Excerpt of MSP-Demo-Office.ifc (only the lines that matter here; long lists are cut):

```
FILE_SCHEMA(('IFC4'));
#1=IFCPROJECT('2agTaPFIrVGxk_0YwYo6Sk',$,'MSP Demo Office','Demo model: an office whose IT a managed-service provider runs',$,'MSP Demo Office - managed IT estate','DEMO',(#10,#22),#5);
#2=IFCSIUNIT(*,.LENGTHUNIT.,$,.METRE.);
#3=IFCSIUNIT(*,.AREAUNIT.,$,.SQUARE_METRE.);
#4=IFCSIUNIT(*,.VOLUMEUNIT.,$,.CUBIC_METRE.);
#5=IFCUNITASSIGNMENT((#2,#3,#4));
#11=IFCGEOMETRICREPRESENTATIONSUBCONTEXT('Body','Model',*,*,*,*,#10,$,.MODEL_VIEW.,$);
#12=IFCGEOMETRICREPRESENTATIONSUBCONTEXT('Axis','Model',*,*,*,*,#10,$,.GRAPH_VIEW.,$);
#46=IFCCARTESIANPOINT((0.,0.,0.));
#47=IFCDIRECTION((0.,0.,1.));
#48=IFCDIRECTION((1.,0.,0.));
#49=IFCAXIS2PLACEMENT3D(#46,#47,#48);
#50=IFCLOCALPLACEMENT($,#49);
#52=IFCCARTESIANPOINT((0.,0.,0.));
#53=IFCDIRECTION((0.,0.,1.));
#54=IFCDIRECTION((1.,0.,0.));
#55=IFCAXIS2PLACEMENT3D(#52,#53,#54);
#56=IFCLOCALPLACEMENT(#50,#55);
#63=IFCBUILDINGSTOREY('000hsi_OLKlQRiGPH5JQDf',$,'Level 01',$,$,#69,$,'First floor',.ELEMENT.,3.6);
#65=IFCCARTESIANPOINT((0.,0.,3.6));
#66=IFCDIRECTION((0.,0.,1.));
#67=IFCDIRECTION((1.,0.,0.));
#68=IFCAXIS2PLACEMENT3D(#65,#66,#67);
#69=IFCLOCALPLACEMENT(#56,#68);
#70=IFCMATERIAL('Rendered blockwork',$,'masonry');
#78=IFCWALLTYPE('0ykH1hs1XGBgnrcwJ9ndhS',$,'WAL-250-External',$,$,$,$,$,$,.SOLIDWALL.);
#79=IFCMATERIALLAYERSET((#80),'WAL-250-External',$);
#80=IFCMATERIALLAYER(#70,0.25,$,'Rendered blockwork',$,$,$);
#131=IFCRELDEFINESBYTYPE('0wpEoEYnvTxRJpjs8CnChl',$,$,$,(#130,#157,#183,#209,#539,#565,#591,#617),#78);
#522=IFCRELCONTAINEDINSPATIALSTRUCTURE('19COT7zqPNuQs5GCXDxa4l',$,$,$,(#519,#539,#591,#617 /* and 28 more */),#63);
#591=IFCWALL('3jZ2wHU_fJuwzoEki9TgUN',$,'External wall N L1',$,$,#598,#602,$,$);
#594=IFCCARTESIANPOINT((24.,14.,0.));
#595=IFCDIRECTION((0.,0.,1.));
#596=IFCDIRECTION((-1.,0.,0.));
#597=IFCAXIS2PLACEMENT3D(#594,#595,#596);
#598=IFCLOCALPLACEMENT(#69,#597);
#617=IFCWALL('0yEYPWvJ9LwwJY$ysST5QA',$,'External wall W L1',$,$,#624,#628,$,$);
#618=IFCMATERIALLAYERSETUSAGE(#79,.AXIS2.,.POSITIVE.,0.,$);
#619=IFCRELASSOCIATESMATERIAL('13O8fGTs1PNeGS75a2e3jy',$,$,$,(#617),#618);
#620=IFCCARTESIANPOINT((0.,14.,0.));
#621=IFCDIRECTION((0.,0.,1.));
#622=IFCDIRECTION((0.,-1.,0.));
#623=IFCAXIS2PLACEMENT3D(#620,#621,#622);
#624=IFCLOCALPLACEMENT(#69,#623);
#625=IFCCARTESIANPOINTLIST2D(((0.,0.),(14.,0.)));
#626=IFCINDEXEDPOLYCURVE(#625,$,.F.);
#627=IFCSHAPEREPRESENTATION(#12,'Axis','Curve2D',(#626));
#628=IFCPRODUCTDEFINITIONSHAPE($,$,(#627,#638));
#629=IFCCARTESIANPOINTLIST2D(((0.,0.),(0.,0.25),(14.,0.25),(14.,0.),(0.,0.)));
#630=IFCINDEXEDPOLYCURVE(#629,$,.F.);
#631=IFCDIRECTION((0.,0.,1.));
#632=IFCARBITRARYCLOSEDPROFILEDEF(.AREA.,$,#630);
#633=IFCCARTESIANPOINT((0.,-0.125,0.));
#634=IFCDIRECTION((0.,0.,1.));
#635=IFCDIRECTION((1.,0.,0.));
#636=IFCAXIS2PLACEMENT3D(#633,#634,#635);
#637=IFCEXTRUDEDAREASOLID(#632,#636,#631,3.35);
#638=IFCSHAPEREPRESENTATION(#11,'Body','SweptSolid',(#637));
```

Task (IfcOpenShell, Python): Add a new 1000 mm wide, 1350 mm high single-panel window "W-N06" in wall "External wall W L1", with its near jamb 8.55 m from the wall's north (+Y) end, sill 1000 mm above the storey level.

```python
import numpy as np
import ifcopenshell
import ifcopenshell.api.feature
import ifcopenshell.api.geometry
import ifcopenshell.api.root
import ifcopenshell.api.spatial
import ifcopenshell.geom
import ifcopenshell.util.element
import ifcopenshell.util.placement
import ifcopenshell.util.representation
import ifcopenshell.util.shape
import ifcopenshell.util.unit

model = ifcopenshell.open("MSP-Demo-Office.ifc")
unit_scale = ifcopenshell.util.unit.calculate_unit_scale(model)
settings = ifcopenshell.geom.settings()


def volume(element):
    """Net volume in cubic metres, openings subtracted."""
    shape = ifcopenshell.geom.create_shape(settings, element)
    return ifcopenshell.util.shape.get_volume(shape.geometry)


wall = model.by_guid("0yEYPWvJ9LwwJY$ysST5QA")
storey = ifcopenshell.util.element.get_container(wall, ifc_class="IfcBuildingStorey")
context = ifcopenshell.util.representation.get_context(model, "Model", "Body", "MODEL_VIEW")
before = volume(wall)

width, height, from_end, sill = 1, 1.35, 8.55, 1  # metres

# The wall runs along its own X axis, and the end named is its -X end.
wall_shape = ifcopenshell.geom.create_shape(settings, wall)
x, y, z = ifcopenshell.util.shape.get_vertices(wall_shape.geometry).T
start = x.min() + from_end
face, thickness = float(y.min()), float(y.max() - y.min())
wall_matrix = ifcopenshell.util.placement.get_local_placement(wall.ObjectPlacement)
level = ifcopenshell.util.placement.get_local_placement(storey.ObjectPlacement)[2, 3]


def in_wall(x, y):
    """Placement at x, y metres in the wall's axes, at sill height."""
    matrix = wall_matrix.copy()
    matrix[:, 3] = wall_matrix @ np.array([x / unit_scale, y / unit_scale, 0.0, 1.0])
    matrix[2, 3] = level + sill / unit_scale
    return matrix


# Opening: a box that overshoots both wall faces by 50 mm.
opening = ifcopenshell.api.root.create_entity(model, ifc_class="IfcOpeningElement", predefined_type="OPENING")
box = ifcopenshell.api.geometry.add_wall_representation(
    model, context=context, length=width, height=height, thickness=thickness + 0.1
)
ifcopenshell.api.geometry.assign_representation(model, product=opening, representation=box)
ifcopenshell.api.geometry.edit_object_placement(model, product=opening, matrix=in_wall(start, face - 0.05), is_si=False)
ifcopenshell.api.feature.add_feature(model, feature=opening, element=wall)

window = ifcopenshell.api.root.create_entity(model, ifc_class="IfcWindow", name="W-N06", predefined_type="WINDOW")
window.OverallWidth, window.OverallHeight = width / unit_scale, height / unit_scale
window.PartitioningType = "SINGLE_PANEL"
body = ifcopenshell.api.geometry.add_window_representation(
    model,
    context=context,
    overall_width=window.OverallWidth,
    overall_height=window.OverallHeight,
    partition_type="SINGLE_PANEL",
)
ifcopenshell.api.geometry.assign_representation(model, product=window, representation=body)
ifcopenshell.api.spatial.assign_container(model, products=[window], relating_structure=storey)
ifcopenshell.api.feature.add_filling(model, opening=opening, element=window)

# Centre the window in the wall's thickness.
ifcopenshell.api.geometry.edit_object_placement(model, product=window, matrix=in_wall(start, face), is_si=False)
window_shape = ifcopenshell.geom.create_shape(settings, window)
depth = ifcopenshell.util.shape.get_vertices(window_shape.geometry)[:, 1]
offset = face + thickness / 2 - (depth.min() + depth.max()) / 2
ifcopenshell.api.geometry.edit_object_placement(model, product=window, matrix=in_wall(start, offset), is_si=False)

after = volume(wall)

print(f"wall volume {before:.3f} -> {after:.3f} m3")

model.write("MSP-Demo-Office_rev.ifc")
```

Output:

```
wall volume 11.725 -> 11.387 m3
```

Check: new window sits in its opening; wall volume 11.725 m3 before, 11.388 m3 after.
